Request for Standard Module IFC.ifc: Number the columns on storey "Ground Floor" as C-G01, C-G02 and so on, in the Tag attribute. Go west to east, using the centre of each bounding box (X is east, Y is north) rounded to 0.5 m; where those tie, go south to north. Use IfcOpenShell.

First a look at what the model holds.

```python
import ifcopenshell
import ifcopenshell.util.element
import ifcopenshell.util.placement

model = ifcopenshell.open("Standard Module IFC.ifc")
print(model.schema)
storey = next(s for s in model.by_type("IfcBuildingStorey") if s.Name == "Ground Floor")
columns = [e for e in ifcopenshell.util.element.get_decomposition(storey) if e.is_a("IfcColumn")]
for e in sorted(columns, key=lambda e: e.id()):
    origin = ifcopenshell.util.placement.get_local_placement(e.ObjectPlacement)[:3, 3]
    print(e.id(), e.Tag, e.Name, origin.round(2) + 0.0, sep=" | ")
```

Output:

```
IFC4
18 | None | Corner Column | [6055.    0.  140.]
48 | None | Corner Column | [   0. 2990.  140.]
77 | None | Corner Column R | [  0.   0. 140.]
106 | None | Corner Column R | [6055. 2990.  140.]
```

```python
import ifcopenshell
import ifcopenshell.geom
import ifcopenshell.util.element
import ifcopenshell.util.shape

model = ifcopenshell.open("Standard Module IFC.ifc")
settings = ifcopenshell.geom.settings()
settings.set("use-world-coords", True)


def centre(element):
    shape = ifcopenshell.geom.create_shape(settings, element)
    return ifcopenshell.util.shape.get_bbox_centroid(shape.geometry)


storey = next(s for s in model.by_type("IfcBuildingStorey") if s.Name == "Ground Floor")
columns = [e for e in ifcopenshell.util.element.get_decomposition(storey) if e.is_a("IfcColumn")]

# Insertion points can sit at a corner or the storey origin, so sort by the geometry (in metres).
centres = {e: centre(e) for e in columns}
columns.sort(key=lambda e: (round(centres[e][0] / 0.5), centres[e][1]))

for i, e in enumerate(columns, start=1):
    number = f"C-G{i:02d}"
    e.Tag = number
    print(e.id(), number)

model.write("Standard Module IFC_v2.ifc")
```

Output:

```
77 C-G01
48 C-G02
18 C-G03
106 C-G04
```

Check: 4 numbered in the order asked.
